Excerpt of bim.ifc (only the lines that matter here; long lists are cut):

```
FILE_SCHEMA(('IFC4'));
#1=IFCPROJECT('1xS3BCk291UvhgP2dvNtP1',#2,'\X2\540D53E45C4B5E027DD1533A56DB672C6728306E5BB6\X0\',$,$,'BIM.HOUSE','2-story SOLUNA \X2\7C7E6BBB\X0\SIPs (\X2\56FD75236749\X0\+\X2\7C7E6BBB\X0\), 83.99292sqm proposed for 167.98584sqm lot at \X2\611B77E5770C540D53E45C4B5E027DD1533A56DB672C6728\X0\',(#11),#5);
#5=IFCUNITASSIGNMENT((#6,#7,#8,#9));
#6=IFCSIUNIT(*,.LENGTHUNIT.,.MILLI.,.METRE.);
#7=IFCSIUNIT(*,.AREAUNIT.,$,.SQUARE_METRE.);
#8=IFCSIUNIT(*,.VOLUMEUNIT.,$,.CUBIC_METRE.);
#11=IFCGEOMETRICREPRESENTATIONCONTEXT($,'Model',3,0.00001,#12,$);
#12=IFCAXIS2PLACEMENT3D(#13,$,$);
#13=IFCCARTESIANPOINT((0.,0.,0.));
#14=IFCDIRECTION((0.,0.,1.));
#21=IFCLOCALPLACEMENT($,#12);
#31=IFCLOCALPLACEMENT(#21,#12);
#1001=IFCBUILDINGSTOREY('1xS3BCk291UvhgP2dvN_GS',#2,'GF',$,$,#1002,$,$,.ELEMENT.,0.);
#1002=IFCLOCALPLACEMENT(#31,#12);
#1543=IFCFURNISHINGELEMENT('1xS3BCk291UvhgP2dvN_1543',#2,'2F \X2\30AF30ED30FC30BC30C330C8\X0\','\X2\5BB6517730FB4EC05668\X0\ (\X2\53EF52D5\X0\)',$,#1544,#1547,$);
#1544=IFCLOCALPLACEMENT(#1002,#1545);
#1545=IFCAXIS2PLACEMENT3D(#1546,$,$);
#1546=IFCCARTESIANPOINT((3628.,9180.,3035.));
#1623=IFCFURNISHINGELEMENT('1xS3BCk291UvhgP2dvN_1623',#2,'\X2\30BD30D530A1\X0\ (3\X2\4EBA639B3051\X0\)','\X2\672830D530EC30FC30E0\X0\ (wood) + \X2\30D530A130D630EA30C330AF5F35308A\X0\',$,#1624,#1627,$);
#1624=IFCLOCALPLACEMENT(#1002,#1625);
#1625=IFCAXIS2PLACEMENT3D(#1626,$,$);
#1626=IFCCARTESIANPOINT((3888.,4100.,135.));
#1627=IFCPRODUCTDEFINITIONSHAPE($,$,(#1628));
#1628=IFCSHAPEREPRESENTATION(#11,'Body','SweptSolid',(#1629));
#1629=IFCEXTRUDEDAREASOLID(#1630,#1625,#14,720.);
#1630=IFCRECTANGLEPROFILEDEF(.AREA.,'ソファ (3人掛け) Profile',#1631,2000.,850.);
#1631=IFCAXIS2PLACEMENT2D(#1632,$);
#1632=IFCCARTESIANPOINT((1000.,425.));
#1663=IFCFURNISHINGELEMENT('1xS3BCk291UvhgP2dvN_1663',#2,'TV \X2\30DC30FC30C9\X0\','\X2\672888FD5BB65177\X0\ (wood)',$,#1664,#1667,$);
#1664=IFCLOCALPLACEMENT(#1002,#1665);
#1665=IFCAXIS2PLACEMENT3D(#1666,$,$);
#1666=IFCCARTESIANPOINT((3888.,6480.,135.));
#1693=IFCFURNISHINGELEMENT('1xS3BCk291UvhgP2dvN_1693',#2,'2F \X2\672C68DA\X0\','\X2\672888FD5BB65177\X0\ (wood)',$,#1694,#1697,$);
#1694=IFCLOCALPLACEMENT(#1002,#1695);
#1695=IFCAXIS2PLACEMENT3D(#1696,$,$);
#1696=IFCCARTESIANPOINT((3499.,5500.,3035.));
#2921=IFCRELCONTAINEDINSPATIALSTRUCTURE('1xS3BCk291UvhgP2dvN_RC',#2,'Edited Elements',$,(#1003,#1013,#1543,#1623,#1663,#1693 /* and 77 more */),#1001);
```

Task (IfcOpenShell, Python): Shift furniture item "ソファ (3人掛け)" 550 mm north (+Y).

```python
import ifcopenshell
import ifcopenshell.api.geometry
import ifcopenshell.util.placement
import ifcopenshell.util.unit

model = ifcopenshell.open("bim.ifc")
unit_scale = ifcopenshell.util.unit.calculate_unit_scale(model)

item = model.by_id(1623)
matrix = ifcopenshell.util.placement.get_local_placement(item.ObjectPlacement)
matrix[1, 3] += 0.55 / unit_scale
ifcopenshell.api.geometry.edit_object_placement(model, product=item, matrix=matrix, is_si=False)

print(ifcopenshell.util.placement.get_local_placement(item.ObjectPlacement).round(3) + 0.0)

model.write("bim-out.ifc")
```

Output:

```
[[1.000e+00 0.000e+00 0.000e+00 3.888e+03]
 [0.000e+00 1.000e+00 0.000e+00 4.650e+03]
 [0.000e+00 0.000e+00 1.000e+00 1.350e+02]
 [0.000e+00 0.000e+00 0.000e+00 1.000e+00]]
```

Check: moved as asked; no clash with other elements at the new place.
